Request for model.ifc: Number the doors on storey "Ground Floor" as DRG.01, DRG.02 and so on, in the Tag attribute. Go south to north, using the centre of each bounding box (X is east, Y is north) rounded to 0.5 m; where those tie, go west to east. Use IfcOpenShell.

First a look at what the model holds.

```python
import ifcopenshell
import ifcopenshell.util.element
import ifcopenshell.util.placement

model = ifcopenshell.open("model.ifc")
print(model.schema)
storey = next(s for s in model.by_type("IfcBuildingStorey") if s.Name == "Ground Floor")
doors = [e for e in ifcopenshell.util.element.get_decomposition(storey) if e.is_a("IfcDoor")]
for e in sorted(doors, key=lambda e: e.id()):
    origin = ifcopenshell.util.placement.get_local_placement(e.ObjectPlacement)[:3, 3]
    print(e.id(), e.Tag, e.Name, origin.round(2) + 0.0, sep=" | ")
```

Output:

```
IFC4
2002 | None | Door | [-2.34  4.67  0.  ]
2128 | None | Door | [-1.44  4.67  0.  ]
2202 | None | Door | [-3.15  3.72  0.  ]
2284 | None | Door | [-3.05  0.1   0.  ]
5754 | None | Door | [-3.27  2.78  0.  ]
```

```python
import ifcopenshell
import ifcopenshell.geom
import ifcopenshell.util.element
import ifcopenshell.util.shape

model = ifcopenshell.open("model.ifc")
settings = ifcopenshell.geom.settings()
settings.set("use-world-coords", True)


def centre(element):
    shape = ifcopenshell.geom.create_shape(settings, element)
    return ifcopenshell.util.shape.get_bbox_centroid(shape.geometry)


storey = next(s for s in model.by_type("IfcBuildingStorey") if s.Name == "Ground Floor")
doors = [e for e in ifcopenshell.util.element.get_decomposition(storey) if e.is_a("IfcDoor")]

# Insertion points can sit at a corner or the storey origin, so sort by the geometry (in metres).
centres = {e: centre(e) for e in doors}
doors.sort(key=lambda e: (round(centres[e][1] / 0.5), centres[e][0]))

for i, e in enumerate(doors, start=1):
    number = f"DRG.{i:02d}"
    e.Tag = number
    print(e.id(), number)

model.write("model_updated.ifc")
```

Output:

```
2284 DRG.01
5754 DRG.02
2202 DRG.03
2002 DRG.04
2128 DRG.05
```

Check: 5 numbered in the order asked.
